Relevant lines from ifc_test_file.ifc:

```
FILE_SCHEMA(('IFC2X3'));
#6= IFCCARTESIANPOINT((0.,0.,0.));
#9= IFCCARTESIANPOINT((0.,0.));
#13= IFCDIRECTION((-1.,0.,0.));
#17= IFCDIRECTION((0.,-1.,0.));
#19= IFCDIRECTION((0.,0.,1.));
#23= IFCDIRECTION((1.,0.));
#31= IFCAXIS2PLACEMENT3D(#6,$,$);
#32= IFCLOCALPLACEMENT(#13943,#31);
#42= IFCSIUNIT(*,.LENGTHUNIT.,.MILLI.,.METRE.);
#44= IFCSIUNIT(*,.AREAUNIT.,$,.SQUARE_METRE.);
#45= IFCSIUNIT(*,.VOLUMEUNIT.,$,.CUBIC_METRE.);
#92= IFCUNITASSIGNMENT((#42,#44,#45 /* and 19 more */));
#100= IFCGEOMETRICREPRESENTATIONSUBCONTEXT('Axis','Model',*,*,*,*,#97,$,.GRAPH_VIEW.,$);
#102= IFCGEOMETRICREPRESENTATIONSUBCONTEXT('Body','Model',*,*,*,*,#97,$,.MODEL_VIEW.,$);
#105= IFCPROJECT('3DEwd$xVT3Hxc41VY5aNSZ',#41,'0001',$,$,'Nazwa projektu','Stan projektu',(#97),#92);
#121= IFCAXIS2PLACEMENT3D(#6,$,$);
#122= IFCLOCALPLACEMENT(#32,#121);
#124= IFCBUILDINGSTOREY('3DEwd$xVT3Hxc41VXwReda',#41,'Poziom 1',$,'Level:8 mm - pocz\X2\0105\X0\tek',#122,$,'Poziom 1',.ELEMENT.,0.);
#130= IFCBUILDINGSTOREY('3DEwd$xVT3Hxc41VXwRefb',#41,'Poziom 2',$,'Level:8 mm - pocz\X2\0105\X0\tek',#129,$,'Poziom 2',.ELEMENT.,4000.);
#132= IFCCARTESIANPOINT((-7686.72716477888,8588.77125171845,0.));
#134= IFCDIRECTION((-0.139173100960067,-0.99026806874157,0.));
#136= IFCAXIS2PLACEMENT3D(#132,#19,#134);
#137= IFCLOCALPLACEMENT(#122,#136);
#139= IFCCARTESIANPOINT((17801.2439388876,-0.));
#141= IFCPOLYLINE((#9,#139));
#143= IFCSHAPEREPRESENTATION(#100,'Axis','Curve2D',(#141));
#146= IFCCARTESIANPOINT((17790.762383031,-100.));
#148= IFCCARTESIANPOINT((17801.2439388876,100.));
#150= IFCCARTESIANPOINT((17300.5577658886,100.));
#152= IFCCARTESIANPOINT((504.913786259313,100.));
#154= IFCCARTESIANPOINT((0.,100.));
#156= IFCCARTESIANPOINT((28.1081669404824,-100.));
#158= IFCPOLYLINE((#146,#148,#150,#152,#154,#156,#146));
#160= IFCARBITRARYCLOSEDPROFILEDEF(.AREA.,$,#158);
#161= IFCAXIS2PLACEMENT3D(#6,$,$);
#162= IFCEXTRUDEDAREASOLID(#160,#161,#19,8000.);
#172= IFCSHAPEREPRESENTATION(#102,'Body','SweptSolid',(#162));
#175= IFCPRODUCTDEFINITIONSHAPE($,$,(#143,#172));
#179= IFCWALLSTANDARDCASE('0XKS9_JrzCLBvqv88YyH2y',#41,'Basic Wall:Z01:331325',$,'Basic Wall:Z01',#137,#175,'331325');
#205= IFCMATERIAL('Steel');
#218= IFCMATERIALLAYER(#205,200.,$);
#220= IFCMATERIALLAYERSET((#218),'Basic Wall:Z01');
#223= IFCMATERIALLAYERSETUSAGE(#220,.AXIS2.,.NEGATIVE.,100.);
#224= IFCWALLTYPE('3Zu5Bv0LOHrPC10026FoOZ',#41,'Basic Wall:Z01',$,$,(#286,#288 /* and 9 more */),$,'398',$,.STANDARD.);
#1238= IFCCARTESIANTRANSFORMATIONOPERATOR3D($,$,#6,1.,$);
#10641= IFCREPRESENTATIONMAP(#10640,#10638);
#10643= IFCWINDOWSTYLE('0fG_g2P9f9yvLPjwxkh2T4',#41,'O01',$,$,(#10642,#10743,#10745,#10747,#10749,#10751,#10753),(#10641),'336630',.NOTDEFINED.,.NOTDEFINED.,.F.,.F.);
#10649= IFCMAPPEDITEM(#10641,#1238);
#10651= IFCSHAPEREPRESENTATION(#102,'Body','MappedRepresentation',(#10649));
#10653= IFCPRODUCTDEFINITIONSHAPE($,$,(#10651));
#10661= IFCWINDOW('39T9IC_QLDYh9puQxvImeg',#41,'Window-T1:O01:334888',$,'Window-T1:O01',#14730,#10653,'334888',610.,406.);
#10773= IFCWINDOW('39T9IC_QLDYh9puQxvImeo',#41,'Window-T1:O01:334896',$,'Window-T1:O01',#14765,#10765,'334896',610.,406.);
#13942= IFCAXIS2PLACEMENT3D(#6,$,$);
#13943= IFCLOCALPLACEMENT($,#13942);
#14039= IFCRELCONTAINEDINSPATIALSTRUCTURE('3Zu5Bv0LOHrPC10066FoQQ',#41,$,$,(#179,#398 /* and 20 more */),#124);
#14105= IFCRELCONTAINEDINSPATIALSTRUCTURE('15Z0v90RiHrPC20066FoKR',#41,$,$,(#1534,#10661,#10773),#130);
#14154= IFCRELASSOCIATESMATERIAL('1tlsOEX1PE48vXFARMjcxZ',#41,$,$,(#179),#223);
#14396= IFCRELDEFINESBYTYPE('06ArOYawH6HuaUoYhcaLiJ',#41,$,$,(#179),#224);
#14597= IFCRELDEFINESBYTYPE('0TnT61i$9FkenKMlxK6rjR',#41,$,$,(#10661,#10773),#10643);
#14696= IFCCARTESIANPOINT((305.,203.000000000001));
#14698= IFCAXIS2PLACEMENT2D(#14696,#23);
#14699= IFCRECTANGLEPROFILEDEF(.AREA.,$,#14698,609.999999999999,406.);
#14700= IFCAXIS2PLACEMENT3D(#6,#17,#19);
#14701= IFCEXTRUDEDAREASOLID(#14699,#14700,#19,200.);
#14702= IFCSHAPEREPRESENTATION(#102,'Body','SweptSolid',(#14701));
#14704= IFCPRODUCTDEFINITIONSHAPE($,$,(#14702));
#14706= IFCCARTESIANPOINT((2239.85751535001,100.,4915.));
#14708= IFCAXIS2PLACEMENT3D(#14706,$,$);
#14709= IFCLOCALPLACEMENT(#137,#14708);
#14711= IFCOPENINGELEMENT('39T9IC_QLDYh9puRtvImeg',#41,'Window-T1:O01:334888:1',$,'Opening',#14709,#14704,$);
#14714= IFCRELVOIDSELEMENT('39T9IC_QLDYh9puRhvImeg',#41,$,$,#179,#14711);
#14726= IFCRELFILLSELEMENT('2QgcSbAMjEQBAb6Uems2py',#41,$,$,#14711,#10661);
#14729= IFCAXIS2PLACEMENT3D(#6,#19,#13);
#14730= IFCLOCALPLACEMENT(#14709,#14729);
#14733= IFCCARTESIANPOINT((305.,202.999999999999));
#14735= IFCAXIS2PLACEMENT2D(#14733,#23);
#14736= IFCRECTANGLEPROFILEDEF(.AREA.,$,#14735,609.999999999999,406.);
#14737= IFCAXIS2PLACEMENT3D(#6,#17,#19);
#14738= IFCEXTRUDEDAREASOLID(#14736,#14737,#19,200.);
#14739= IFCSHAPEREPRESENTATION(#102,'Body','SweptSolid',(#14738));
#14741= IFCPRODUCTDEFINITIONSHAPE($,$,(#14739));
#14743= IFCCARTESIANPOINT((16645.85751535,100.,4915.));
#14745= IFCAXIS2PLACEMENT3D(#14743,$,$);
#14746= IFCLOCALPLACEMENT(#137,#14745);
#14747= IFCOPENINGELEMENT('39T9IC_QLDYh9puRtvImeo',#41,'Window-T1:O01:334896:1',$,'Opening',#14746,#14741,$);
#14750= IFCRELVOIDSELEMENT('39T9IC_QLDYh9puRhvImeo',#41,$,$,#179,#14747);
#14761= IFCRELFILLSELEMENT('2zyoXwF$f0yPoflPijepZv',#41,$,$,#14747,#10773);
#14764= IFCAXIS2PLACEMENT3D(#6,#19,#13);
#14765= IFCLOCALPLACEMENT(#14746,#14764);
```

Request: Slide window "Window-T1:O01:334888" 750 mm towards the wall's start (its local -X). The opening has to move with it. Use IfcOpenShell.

```python
import ifcopenshell
import ifcopenshell.api.geometry
import ifcopenshell.util.placement

model = ifcopenshell.open("ifc_test_file.ifc")

window = model.by_guid("39T9IC_QLDYh9puQxvImeg")
opening = window.FillsVoids[0].RelatingOpeningElement
wall = opening.VoidsElements[0].RelatingBuildingElement

wall_matrix = ifcopenshell.util.placement.get_local_placement(wall.ObjectPlacement)
shift = wall_matrix[:3, 0] * -750.0
before = ifcopenshell.util.placement.get_local_placement(window.ObjectPlacement)[:3, 3].copy()

# The window is placed relative to its opening, so it follows when the opening moves.
matrix = ifcopenshell.util.placement.get_local_placement(opening.ObjectPlacement)
matrix[:3, 3] += shift
ifcopenshell.api.geometry.edit_object_placement(
    model, product=opening, matrix=matrix, is_si=False, should_transform_children=True
)

after = ifcopenshell.util.placement.get_local_placement(window.ObjectPlacement)[:3, 3]
print("window moved by", (after - before).round(3) + 0.0)

model.write("ifc_test_file_updated.ifc")
```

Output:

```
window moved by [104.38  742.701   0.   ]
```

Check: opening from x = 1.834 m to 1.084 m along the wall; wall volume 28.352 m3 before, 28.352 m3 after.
